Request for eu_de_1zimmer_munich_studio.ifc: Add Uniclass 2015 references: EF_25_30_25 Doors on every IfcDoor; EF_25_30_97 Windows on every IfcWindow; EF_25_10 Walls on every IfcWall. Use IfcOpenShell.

First a look at what the model holds.

```python
import ifcopenshell

model = ifcopenshell.open("eu_de_1zimmer_munich_studio.ifc")
print(model.schema)
print("classifications:", [c.Name for c in model.by_type("IfcClassification")])
for ifc_class in ("IfcDoor", "IfcRoof", "IfcStair", "IfcWall", "IfcWindow"):
    print(ifc_class, len(model.by_type(ifc_class)))
```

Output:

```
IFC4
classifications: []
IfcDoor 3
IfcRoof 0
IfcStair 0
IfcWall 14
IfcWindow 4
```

```python
import ifcopenshell
import ifcopenshell.api.classification

model = ifcopenshell.open("eu_de_1zimmer_munich_studio.ifc")

system = ifcopenshell.api.classification.add_classification(model, classification="Uniclass 2015")

codes = {
    "IfcDoor": ("EF_25_30_25", "Doors"),
    "IfcWindow": ("EF_25_30_97", "Windows"),
    "IfcWall": ("EF_25_10", "Walls"),
}
for ifc_class, (code, name) in codes.items():
    products = model.by_type(ifc_class)
    ifcopenshell.api.classification.add_reference(
        model, products=products, classification=system, identification=code, name=name
    )
    print(code, len(products))

model.write("eu_de_1zimmer_munich_studio_updated.ifc")
```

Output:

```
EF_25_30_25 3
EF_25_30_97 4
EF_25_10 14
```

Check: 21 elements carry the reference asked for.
